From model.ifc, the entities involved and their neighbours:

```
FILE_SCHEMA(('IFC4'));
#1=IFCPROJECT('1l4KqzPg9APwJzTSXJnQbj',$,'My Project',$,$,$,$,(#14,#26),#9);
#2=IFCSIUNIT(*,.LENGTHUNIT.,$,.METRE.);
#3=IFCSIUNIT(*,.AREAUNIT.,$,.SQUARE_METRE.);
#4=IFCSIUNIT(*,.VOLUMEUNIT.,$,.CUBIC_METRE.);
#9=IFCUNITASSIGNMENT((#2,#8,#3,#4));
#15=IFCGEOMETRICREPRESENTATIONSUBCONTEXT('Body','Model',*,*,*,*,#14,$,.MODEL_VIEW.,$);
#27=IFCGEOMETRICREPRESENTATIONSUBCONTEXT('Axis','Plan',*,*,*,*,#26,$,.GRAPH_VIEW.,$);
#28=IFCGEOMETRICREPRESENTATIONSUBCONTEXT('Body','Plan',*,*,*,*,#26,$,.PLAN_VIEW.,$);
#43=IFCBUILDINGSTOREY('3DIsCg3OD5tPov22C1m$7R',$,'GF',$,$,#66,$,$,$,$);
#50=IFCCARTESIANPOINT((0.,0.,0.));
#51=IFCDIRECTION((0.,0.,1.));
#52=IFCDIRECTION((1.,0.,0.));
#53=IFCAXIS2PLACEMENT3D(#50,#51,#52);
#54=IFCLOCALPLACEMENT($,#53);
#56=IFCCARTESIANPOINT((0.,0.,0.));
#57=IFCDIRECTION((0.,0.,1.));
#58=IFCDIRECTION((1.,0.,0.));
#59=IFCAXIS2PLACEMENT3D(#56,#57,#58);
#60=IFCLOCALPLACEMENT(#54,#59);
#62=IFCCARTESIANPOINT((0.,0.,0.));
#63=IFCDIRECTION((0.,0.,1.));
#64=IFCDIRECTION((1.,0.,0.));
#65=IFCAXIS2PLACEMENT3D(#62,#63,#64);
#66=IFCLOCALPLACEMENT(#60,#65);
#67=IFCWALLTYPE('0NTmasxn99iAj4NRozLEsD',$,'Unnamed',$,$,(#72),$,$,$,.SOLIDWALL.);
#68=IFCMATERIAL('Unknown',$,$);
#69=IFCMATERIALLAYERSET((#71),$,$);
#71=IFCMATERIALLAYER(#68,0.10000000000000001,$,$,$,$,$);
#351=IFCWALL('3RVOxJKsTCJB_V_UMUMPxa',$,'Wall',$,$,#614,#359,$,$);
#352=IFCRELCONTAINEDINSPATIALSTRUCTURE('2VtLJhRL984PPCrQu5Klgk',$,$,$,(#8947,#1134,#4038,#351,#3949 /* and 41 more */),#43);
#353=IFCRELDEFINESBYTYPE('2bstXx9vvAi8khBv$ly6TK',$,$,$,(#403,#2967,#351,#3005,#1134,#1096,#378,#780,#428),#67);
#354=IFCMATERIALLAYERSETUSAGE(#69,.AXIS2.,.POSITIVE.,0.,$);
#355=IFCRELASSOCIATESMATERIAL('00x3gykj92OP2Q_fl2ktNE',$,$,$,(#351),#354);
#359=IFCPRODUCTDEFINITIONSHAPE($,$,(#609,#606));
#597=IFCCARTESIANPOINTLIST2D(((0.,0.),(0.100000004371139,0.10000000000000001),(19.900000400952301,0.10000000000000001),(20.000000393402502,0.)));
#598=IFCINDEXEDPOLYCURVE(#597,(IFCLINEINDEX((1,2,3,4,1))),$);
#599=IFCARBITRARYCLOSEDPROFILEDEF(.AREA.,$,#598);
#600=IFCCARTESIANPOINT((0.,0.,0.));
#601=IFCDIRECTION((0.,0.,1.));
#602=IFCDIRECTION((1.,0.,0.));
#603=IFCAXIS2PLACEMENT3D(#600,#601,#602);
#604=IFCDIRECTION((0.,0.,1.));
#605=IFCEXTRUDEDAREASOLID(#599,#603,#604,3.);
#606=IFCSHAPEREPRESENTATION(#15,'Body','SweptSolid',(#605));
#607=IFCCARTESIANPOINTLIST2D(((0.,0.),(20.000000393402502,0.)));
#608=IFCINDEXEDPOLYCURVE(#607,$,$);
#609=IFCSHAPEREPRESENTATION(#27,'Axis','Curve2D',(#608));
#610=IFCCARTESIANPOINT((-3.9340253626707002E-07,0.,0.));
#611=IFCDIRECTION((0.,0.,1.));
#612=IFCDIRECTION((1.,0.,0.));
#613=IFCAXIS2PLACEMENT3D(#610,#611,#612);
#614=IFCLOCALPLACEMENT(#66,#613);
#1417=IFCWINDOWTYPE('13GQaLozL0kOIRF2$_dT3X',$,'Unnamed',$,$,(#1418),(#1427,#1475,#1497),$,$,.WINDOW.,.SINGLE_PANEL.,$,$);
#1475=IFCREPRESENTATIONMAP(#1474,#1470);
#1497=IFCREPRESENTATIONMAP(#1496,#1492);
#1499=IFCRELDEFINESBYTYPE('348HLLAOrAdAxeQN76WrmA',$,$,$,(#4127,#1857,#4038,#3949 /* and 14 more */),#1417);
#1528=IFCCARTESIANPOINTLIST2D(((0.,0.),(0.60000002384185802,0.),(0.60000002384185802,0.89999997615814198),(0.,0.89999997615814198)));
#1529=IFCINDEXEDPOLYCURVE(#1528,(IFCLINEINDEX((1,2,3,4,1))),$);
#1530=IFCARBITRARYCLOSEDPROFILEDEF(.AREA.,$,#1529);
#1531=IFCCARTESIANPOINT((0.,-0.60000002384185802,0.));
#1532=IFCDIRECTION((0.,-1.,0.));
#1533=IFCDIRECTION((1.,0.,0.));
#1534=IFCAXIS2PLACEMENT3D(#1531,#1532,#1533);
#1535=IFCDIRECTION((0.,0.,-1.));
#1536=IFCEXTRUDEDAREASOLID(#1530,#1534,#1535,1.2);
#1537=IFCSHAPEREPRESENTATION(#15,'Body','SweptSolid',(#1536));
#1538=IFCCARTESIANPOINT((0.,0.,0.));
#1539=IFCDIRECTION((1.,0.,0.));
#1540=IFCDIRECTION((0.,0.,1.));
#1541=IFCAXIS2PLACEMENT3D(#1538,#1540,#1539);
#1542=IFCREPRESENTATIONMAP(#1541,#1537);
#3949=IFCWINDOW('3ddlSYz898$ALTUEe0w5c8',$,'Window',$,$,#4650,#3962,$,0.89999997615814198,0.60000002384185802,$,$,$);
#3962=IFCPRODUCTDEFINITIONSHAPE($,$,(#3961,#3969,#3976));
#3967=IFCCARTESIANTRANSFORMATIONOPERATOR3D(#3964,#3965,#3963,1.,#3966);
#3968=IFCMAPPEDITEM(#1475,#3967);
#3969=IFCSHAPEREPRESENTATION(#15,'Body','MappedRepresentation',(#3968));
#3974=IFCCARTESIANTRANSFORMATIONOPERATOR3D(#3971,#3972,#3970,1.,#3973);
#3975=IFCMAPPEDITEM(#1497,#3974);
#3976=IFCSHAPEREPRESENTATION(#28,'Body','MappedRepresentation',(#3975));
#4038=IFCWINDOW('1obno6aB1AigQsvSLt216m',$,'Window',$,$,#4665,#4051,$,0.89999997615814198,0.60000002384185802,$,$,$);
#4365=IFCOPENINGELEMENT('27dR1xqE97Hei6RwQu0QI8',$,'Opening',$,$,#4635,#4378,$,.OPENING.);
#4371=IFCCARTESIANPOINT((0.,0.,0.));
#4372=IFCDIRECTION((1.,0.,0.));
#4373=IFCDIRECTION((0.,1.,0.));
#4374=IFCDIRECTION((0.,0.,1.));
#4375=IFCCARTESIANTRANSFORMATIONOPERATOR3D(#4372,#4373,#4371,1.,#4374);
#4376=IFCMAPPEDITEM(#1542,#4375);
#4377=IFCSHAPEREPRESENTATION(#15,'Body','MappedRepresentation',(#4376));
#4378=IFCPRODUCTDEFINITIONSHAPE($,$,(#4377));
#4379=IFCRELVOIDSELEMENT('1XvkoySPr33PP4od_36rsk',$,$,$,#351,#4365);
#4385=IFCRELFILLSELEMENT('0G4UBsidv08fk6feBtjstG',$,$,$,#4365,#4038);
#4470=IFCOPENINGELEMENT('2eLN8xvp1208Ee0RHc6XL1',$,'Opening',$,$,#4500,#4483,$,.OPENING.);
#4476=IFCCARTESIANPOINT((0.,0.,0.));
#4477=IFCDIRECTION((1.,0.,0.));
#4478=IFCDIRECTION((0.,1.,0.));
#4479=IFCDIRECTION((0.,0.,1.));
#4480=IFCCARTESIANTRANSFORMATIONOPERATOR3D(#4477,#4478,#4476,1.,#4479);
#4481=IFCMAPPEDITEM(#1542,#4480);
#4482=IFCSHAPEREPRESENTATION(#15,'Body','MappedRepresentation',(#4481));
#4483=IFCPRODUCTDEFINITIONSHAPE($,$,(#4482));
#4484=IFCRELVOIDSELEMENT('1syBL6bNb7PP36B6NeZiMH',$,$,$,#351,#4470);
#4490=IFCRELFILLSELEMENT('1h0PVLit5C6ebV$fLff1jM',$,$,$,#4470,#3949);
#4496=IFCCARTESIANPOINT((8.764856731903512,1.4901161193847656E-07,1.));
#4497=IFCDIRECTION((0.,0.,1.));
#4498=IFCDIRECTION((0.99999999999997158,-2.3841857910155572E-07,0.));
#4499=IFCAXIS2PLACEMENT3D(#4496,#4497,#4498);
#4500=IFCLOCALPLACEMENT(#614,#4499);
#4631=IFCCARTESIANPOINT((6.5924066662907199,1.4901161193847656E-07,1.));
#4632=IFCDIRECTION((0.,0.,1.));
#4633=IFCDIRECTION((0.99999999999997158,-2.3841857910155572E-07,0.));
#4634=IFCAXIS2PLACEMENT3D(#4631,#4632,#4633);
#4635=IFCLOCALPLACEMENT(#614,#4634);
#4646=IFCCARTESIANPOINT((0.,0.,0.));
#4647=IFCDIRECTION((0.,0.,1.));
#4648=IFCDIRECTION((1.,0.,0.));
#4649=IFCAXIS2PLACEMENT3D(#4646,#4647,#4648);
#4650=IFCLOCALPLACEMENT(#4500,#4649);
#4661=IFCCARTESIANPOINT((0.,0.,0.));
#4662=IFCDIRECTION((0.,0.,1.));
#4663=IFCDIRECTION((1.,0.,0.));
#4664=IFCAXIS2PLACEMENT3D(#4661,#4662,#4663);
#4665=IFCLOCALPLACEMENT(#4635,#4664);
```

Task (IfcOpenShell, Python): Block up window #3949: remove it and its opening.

```python
import ifcopenshell
import ifcopenshell.api.feature
import ifcopenshell.api.root
import ifcopenshell.geom
import ifcopenshell.util.shape

model = ifcopenshell.open("model.ifc")
settings = ifcopenshell.geom.settings()


def volume(element):
    """Net volume in cubic metres, openings subtracted."""
    shape = ifcopenshell.geom.create_shape(settings, element)
    return ifcopenshell.util.shape.get_volume(shape.geometry)


window = model.by_guid("3ddlSYz898$ALTUEe0w5c8")
opening = window.FillsVoids[0].RelatingOpeningElement
wall = opening.VoidsElements[0].RelatingBuildingElement
before = volume(wall)

ifcopenshell.api.root.remove_product(model, product=window)
ifcopenshell.api.feature.remove_feature(model, feature=opening)

after = volume(wall)

print(f"wall volume {before:.3f} -> {after:.3f} m3")

model.write("model_rev.ifc")
```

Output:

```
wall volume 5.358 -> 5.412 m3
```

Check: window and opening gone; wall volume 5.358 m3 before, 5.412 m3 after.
